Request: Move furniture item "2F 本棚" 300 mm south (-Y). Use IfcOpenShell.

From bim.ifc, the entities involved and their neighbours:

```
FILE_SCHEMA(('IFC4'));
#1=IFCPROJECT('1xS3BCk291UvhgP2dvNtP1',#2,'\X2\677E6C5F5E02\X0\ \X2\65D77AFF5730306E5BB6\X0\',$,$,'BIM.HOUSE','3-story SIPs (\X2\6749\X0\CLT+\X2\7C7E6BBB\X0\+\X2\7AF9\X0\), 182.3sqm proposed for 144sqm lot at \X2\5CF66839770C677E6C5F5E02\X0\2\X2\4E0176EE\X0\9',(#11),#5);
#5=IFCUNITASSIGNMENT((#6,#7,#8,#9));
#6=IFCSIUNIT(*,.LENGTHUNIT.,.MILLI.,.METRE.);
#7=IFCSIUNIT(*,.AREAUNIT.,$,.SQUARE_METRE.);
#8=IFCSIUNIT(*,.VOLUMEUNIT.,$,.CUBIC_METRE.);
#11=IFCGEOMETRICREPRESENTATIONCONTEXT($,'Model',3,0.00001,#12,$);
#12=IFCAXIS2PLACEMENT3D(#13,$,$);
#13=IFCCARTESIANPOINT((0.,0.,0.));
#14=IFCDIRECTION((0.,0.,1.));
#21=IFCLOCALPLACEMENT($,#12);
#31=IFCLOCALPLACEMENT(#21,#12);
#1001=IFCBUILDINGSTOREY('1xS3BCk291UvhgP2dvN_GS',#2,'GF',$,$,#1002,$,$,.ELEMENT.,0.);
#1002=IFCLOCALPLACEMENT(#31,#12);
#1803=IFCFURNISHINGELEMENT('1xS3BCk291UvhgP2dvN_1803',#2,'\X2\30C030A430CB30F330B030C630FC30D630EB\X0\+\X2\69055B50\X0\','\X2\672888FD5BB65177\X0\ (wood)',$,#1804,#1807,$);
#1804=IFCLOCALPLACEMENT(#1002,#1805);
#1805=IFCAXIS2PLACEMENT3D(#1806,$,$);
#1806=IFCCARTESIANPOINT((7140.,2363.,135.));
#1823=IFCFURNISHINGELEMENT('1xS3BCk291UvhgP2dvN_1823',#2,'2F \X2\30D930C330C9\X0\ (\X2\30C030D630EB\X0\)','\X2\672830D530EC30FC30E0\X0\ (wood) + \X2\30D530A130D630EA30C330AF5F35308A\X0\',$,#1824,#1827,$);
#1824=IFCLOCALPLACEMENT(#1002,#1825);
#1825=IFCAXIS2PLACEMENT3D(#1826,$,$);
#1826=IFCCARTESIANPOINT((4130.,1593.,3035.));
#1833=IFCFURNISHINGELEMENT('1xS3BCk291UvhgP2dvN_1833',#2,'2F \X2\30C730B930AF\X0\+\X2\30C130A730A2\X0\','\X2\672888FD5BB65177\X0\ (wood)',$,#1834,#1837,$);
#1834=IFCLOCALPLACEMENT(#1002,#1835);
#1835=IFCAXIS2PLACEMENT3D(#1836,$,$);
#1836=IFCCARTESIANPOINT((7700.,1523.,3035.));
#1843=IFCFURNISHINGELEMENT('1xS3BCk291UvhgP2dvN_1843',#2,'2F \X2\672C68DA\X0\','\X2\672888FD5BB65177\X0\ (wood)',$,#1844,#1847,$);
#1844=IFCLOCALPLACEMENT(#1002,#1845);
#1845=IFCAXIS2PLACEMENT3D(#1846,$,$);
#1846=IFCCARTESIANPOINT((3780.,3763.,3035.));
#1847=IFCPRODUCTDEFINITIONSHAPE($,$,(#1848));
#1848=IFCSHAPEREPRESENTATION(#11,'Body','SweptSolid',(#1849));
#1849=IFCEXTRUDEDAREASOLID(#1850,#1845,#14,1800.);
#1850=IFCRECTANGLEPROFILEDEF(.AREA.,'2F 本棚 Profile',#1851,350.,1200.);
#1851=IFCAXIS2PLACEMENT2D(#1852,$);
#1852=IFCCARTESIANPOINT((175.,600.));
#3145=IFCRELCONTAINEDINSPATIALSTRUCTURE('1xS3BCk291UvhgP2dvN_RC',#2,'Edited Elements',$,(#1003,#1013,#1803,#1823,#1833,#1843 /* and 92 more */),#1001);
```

```python
import ifcopenshell
import ifcopenshell.api.geometry
import ifcopenshell.util.placement
import ifcopenshell.util.unit

model = ifcopenshell.open("bim.ifc")
unit_scale = ifcopenshell.util.unit.calculate_unit_scale(model)

item = model.by_guid("1xS3BCk291UvhgP2dvN_1843")
matrix = ifcopenshell.util.placement.get_local_placement(item.ObjectPlacement)
matrix[1, 3] -= 0.3 / unit_scale
ifcopenshell.api.geometry.edit_object_placement(model, product=item, matrix=matrix, is_si=False)

print(ifcopenshell.util.placement.get_local_placement(item.ObjectPlacement).round(3) + 0.0)

model.write("bim_edited.ifc")
```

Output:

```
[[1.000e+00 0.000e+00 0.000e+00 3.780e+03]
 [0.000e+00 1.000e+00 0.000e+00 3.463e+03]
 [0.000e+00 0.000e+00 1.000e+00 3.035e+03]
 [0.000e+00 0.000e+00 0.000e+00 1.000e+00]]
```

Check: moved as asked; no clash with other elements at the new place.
